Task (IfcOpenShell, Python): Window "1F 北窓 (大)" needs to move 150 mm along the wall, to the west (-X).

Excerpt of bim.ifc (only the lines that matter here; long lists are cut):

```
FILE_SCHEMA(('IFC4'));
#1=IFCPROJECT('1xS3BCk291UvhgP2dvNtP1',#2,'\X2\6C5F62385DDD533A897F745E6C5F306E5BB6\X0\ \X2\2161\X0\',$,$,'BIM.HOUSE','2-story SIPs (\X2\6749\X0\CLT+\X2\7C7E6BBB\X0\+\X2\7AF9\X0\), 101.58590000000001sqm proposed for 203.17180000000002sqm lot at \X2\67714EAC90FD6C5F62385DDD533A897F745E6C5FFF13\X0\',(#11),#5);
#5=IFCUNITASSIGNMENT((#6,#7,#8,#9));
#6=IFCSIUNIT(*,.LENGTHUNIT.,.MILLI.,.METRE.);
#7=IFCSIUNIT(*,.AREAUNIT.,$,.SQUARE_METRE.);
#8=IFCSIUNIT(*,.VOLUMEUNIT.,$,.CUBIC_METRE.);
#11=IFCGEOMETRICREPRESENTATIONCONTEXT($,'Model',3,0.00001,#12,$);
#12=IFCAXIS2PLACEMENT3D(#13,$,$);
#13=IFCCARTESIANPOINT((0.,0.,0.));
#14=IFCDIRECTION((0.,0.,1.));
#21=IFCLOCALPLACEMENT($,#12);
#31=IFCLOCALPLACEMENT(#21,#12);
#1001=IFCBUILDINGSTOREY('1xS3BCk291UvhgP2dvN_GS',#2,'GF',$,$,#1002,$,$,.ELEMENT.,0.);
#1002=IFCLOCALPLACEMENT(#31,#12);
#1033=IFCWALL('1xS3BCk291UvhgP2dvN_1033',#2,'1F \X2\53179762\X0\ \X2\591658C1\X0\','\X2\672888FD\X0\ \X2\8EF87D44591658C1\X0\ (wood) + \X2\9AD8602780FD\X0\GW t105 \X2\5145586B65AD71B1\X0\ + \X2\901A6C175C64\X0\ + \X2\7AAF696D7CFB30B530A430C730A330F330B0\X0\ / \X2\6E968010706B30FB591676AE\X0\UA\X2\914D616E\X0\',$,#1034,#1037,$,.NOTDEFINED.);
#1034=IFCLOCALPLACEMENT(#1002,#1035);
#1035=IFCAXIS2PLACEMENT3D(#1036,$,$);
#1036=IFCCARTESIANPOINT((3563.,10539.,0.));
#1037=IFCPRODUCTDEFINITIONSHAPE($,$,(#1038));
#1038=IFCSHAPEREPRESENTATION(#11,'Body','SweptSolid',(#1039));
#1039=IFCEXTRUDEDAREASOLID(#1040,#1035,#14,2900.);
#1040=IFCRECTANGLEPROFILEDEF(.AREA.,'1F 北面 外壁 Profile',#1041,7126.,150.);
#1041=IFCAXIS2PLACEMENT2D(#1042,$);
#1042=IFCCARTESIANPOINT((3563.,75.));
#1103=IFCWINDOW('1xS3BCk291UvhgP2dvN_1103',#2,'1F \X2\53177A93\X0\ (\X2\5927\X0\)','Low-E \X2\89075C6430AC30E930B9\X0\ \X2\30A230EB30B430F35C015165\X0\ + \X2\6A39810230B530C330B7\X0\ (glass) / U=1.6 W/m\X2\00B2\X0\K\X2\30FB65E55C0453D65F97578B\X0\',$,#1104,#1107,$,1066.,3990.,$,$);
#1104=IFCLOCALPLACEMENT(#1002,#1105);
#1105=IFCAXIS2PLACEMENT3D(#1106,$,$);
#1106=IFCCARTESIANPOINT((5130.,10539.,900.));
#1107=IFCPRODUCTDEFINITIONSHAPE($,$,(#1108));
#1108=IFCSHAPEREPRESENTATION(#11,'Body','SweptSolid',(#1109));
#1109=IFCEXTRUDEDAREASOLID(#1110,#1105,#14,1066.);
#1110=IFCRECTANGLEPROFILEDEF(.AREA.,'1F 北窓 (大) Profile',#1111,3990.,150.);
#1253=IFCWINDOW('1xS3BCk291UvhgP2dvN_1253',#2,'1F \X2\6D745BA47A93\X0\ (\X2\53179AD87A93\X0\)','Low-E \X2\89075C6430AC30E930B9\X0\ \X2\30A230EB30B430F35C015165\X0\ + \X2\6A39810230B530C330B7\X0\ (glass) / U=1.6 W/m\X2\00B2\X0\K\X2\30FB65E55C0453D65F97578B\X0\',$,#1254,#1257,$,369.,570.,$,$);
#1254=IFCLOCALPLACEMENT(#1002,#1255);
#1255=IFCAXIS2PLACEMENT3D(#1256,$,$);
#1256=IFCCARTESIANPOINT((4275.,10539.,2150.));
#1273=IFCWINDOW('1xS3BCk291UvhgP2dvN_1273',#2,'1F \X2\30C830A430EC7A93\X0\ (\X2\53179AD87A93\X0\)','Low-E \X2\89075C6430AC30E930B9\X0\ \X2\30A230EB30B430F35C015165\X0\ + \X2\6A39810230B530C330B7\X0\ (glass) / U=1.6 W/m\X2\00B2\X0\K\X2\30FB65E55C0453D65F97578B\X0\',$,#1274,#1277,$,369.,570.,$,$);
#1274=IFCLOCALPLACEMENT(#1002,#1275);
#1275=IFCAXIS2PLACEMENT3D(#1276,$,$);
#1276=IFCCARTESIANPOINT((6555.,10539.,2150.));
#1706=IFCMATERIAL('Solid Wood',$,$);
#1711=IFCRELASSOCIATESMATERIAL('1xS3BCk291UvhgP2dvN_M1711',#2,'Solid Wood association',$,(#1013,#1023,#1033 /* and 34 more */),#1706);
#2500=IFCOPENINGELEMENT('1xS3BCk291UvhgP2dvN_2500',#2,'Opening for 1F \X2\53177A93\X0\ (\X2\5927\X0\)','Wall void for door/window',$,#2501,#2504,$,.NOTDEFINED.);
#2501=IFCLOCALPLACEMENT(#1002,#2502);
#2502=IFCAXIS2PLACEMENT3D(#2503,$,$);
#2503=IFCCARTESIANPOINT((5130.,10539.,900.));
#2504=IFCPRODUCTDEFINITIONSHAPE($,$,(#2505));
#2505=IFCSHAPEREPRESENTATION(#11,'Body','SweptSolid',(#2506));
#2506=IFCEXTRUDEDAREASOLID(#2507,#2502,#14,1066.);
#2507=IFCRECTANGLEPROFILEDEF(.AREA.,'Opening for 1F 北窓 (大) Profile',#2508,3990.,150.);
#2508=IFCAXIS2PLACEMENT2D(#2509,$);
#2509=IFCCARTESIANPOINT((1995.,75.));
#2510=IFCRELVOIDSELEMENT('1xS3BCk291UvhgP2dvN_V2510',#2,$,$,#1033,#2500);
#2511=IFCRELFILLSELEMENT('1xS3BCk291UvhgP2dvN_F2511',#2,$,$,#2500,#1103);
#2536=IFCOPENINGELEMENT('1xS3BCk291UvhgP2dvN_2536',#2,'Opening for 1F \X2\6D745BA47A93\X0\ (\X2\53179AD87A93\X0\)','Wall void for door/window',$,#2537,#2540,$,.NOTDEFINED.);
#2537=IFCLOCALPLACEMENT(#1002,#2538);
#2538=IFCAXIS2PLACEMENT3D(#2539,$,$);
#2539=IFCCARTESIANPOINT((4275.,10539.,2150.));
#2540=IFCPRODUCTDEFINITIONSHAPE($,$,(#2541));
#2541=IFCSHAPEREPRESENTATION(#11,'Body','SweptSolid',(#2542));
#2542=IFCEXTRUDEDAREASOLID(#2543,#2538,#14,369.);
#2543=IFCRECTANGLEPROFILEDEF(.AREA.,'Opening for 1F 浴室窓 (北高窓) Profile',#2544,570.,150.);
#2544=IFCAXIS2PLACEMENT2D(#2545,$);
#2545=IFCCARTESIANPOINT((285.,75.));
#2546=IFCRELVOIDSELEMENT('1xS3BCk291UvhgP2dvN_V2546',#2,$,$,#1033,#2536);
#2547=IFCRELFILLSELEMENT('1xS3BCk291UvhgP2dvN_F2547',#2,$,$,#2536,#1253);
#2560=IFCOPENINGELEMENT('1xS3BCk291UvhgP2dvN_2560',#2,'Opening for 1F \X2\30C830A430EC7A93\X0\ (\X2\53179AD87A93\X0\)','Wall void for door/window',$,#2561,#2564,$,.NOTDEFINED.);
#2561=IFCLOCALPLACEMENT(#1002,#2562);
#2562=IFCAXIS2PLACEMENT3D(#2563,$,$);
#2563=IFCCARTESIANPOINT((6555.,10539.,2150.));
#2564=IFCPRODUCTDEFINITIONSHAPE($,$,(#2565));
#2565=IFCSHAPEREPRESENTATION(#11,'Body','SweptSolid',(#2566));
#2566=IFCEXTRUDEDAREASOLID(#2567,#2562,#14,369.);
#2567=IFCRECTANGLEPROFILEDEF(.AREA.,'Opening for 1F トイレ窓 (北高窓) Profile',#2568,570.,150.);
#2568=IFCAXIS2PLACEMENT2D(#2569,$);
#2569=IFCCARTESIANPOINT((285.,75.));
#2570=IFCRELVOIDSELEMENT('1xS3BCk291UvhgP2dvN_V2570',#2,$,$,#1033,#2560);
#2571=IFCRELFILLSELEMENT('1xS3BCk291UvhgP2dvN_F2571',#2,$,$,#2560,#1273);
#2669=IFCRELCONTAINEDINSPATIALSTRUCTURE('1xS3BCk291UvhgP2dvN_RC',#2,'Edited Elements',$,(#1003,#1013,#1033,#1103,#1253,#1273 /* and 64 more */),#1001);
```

```python
import ifcopenshell
import ifcopenshell.api.geometry
import ifcopenshell.util.placement
import ifcopenshell.util.unit

model = ifcopenshell.open("bim.ifc")
unit_scale = ifcopenshell.util.unit.calculate_unit_scale(model)

window = model.by_id(1103)
opening = window.FillsVoids[0].RelatingOpeningElement
wall = opening.VoidsElements[0].RelatingBuildingElement

wall_matrix = ifcopenshell.util.placement.get_local_placement(wall.ObjectPlacement)
shift = wall_matrix[:3, 0] * -0.15 / unit_scale
before = ifcopenshell.util.placement.get_local_placement(window.ObjectPlacement)[:3, 3].copy()

# The window is not placed relative to its opening, so move both.
for product in (opening, window):
    matrix = ifcopenshell.util.placement.get_local_placement(product.ObjectPlacement)
    matrix[:3, 3] += shift
    ifcopenshell.api.geometry.edit_object_placement(model, product=product, matrix=matrix, is_si=False)

after = ifcopenshell.util.placement.get_local_placement(window.ObjectPlacement)[:3, 3]
print("window moved by", (after - before).round(3) + 0.0)

model.write("bim_edited.ifc")
```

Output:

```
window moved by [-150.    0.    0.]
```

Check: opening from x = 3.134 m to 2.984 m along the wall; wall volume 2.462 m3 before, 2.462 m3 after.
